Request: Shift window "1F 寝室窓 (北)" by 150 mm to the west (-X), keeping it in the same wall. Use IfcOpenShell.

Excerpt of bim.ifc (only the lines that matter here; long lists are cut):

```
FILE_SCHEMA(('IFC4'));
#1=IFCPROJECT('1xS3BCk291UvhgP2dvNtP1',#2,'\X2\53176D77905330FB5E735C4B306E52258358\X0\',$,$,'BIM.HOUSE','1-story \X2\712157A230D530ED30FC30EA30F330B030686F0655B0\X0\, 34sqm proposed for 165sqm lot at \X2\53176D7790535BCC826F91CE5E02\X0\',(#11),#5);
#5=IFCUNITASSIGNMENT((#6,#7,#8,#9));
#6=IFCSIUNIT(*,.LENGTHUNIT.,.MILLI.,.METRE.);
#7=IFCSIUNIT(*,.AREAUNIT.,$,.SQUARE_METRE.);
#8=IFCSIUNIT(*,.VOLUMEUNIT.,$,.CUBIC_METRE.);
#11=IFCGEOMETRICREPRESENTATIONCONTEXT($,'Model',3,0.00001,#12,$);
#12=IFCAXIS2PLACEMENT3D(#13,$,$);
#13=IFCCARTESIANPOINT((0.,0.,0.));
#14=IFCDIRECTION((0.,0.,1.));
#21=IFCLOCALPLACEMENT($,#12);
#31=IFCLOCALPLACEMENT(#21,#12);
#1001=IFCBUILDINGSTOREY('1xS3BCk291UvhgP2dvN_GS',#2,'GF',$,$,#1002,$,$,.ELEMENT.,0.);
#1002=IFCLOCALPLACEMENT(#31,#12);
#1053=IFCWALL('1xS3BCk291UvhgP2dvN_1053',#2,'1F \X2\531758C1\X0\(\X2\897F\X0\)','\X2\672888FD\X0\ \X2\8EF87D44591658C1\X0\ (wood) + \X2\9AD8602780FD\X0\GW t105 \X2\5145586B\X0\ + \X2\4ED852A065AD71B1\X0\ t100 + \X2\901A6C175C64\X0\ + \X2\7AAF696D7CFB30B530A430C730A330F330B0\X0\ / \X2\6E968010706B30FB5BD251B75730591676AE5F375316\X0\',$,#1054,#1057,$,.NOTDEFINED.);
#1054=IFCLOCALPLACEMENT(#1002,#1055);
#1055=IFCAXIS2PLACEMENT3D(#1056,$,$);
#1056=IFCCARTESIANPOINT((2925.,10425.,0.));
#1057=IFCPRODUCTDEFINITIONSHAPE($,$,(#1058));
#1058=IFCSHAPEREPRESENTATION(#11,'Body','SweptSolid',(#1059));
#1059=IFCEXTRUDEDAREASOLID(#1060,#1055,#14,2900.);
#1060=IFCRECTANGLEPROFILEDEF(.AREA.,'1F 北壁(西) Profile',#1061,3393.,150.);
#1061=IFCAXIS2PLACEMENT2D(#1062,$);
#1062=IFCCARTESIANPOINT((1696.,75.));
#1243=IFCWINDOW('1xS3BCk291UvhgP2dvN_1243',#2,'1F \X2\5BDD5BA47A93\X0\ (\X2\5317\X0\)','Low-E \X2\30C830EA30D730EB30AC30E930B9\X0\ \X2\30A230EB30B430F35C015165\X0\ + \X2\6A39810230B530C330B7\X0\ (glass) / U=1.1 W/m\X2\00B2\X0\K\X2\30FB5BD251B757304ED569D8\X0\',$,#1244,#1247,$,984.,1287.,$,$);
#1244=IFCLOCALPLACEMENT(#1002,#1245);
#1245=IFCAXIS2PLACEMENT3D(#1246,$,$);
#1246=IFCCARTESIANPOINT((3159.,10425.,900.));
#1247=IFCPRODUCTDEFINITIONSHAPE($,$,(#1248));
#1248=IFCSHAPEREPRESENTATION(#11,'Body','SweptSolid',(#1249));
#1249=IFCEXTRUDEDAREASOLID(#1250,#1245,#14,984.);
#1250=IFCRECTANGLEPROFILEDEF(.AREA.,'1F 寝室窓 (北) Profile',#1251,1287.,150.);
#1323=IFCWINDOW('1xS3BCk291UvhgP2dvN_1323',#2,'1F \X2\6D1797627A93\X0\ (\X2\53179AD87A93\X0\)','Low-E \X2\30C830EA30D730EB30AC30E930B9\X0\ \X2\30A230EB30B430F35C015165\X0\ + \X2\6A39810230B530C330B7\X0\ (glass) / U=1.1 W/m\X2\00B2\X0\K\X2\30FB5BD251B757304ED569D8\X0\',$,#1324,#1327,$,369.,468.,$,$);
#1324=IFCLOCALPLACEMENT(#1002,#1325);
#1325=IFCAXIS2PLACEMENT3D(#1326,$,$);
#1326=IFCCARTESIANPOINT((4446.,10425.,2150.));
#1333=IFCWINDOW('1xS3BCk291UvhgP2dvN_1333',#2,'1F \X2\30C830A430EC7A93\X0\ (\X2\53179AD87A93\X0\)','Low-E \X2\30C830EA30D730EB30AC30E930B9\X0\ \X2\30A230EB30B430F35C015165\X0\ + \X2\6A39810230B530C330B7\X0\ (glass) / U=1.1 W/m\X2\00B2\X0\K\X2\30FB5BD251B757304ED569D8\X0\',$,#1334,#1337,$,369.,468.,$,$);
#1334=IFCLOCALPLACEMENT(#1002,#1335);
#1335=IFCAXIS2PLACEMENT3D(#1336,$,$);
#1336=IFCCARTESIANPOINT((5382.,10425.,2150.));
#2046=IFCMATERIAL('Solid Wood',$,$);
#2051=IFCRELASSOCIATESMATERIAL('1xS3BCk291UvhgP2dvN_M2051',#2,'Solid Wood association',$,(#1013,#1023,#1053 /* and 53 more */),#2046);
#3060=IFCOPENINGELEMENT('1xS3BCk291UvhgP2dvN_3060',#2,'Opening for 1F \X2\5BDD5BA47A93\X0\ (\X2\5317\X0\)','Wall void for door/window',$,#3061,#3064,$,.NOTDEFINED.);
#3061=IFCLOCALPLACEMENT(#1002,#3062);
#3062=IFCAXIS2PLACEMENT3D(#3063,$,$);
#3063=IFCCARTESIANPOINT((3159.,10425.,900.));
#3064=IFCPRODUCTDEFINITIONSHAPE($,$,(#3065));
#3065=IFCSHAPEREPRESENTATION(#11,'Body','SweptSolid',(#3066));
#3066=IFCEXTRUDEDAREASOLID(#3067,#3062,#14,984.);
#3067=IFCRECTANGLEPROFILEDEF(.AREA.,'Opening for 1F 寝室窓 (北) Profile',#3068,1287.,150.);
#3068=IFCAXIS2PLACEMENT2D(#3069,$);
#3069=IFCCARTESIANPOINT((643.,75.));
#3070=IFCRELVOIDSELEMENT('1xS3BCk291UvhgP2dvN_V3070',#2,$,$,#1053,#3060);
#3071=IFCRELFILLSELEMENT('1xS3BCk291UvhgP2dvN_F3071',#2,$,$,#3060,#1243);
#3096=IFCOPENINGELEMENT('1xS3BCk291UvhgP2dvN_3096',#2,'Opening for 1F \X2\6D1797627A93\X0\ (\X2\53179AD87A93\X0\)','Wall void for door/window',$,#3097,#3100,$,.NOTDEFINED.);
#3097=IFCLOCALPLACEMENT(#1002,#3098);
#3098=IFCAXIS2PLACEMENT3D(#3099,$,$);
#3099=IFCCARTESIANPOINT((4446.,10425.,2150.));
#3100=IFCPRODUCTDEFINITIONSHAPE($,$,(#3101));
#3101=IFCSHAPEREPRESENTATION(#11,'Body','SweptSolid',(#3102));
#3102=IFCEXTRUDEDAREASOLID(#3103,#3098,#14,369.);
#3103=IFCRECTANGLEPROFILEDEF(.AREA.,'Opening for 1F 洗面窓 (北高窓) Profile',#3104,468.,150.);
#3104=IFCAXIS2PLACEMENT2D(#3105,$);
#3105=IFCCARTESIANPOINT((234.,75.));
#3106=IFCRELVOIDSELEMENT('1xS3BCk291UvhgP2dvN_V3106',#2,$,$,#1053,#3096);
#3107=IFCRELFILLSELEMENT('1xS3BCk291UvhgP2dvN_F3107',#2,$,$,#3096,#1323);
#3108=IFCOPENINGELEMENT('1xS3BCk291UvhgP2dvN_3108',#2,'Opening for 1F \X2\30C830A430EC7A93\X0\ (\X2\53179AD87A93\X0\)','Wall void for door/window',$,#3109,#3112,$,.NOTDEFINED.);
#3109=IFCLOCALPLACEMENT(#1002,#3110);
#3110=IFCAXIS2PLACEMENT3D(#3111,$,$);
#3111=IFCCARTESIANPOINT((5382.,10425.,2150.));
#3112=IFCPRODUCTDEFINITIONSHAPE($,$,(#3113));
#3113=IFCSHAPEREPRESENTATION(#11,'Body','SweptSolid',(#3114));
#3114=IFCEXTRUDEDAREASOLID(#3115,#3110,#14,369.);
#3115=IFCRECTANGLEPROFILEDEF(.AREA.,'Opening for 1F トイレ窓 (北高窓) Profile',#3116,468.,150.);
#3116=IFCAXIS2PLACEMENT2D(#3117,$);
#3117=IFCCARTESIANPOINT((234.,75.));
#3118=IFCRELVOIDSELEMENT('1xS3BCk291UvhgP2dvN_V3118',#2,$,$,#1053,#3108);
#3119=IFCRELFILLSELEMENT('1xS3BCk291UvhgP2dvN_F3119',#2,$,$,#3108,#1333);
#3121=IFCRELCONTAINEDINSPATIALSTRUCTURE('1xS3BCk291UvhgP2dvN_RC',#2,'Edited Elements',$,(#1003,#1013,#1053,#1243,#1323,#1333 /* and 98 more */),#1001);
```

```python
import ifcopenshell
import ifcopenshell.api.geometry
import ifcopenshell.util.placement
import ifcopenshell.util.unit

model = ifcopenshell.open("bim.ifc")
unit_scale = ifcopenshell.util.unit.calculate_unit_scale(model)

window = model.by_guid("1xS3BCk291UvhgP2dvN_1243")
opening = window.FillsVoids[0].RelatingOpeningElement
wall = opening.VoidsElements[0].RelatingBuildingElement

wall_matrix = ifcopenshell.util.placement.get_local_placement(wall.ObjectPlacement)
shift = wall_matrix[:3, 0] * -0.15 / unit_scale
before = ifcopenshell.util.placement.get_local_placement(window.ObjectPlacement)[:3, 3].copy()

# The window is not placed relative to its opening, so move both.
for product in (opening, window):
    matrix = ifcopenshell.util.placement.get_local_placement(product.ObjectPlacement)
    matrix[:3, 3] += shift
    ifcopenshell.api.geometry.edit_object_placement(model, product=product, matrix=matrix, is_si=False)

after = ifcopenshell.util.placement.get_local_placement(window.ObjectPlacement)[:3, 3]
print("window moved by", (after - before).round(3) + 0.0)

model.write("bim_updated.ifc")
```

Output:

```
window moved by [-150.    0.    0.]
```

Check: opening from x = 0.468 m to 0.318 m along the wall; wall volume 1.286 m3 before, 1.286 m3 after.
